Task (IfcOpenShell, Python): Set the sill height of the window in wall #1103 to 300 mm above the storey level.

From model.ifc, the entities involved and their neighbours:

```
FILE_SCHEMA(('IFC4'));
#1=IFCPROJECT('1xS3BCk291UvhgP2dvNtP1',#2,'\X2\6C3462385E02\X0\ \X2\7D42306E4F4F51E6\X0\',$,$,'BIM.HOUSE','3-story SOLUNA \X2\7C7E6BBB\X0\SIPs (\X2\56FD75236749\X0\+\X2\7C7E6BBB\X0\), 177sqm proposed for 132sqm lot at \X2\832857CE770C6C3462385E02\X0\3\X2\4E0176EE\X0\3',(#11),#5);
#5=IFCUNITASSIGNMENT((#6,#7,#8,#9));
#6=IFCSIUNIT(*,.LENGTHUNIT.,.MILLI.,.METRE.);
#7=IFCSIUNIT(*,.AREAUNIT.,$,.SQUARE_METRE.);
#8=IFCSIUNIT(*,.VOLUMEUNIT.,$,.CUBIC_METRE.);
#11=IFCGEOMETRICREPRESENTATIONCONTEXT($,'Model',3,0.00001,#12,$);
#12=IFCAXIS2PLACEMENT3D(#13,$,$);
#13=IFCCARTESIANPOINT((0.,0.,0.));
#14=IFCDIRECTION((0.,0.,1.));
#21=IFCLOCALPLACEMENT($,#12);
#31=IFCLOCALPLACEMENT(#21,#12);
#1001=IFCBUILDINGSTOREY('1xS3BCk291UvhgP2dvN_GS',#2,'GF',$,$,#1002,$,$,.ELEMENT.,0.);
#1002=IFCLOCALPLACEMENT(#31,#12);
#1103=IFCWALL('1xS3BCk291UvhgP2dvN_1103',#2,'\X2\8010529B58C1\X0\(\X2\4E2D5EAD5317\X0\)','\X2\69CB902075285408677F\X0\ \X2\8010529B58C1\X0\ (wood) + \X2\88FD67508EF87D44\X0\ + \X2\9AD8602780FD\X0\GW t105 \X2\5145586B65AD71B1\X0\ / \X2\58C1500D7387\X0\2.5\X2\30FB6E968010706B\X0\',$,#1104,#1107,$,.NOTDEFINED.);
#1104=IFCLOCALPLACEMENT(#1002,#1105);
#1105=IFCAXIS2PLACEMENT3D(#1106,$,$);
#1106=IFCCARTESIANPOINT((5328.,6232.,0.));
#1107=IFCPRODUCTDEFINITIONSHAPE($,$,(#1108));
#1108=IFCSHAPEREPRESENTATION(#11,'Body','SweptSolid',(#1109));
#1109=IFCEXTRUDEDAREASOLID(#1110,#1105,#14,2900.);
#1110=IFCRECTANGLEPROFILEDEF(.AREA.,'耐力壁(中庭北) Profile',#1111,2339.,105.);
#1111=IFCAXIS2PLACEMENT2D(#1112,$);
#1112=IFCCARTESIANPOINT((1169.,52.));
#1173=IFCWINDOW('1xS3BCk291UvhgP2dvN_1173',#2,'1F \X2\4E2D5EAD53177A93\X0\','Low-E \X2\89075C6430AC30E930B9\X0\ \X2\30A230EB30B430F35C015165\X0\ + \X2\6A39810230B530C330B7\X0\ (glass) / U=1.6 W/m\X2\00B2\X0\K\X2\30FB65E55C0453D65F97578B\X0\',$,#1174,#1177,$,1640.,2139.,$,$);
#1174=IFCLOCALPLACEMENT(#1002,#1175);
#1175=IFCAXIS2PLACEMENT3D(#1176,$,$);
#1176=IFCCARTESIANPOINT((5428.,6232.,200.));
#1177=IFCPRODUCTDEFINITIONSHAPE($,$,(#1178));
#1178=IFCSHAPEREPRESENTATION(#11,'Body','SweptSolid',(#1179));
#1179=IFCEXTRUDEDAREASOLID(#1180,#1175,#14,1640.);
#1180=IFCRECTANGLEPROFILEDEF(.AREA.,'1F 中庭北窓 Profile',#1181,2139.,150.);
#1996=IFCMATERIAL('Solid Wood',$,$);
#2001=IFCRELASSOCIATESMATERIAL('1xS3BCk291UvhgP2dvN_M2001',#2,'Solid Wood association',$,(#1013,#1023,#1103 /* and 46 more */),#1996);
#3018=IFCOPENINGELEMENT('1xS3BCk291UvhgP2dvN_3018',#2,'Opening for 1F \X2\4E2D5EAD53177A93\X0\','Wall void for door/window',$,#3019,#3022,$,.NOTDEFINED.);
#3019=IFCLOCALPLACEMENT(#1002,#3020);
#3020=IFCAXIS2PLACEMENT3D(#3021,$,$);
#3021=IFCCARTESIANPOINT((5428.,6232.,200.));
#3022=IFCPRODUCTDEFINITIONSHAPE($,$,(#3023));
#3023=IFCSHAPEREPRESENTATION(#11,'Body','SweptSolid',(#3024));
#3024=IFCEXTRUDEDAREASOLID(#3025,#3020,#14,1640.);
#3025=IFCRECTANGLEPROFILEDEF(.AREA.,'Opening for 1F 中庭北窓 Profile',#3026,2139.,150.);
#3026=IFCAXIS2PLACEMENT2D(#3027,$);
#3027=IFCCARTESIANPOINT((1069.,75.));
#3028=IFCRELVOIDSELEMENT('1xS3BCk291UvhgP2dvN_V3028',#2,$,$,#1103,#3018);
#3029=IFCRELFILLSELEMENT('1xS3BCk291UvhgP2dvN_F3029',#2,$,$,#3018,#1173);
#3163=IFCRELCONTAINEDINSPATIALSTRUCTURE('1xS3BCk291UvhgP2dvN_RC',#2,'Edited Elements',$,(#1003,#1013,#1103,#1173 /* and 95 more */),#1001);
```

```python
import numpy as np
import ifcopenshell
import ifcopenshell.api.geometry
import ifcopenshell.geom
import ifcopenshell.util.element
import ifcopenshell.util.placement
import ifcopenshell.util.shape
import ifcopenshell.util.unit

model = ifcopenshell.open("model.ifc")
unit_scale = ifcopenshell.util.unit.calculate_unit_scale(model)

window = model.by_id(1173)
opening = window.FillsVoids[0].RelatingOpeningElement
storey = ifcopenshell.util.element.get_container(window, ifc_class="IfcBuildingStorey")
level = ifcopenshell.util.placement.get_local_placement(storey.ObjectPlacement)[2, 3]

# The opening's origin need not be at the sill, so measure its lowest point.
shape = ifcopenshell.geom.create_shape(ifcopenshell.geom.settings(), opening)
bottom = ifcopenshell.util.shape.get_shape_bottom_elevation(shape, shape.geometry) / unit_scale
dz = level + 300.0 - bottom

shift = np.array([0.0, 0.0, dz])
# The window is not placed relative to its opening, so move both.
for product in (opening, window):
    matrix = ifcopenshell.util.placement.get_local_placement(product.ObjectPlacement)
    matrix[:3, 3] += shift
    ifcopenshell.api.geometry.edit_object_placement(model, product=product, matrix=matrix, is_si=False)

print(f"moved by {dz * unit_scale:+.3f} m")

model.write("model_v2.ifc")
```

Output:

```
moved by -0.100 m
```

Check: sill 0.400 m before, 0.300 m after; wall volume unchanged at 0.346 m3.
